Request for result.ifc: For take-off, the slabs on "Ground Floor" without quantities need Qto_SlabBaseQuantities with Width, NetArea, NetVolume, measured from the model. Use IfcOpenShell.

First a look at what the model holds.

```python
import ifcopenshell
import ifcopenshell.util.element
import ifcopenshell.util.unit

model = ifcopenshell.open("result.ifc")
print(model.schema)
for unit_type in ("LENGTHUNIT", "AREAUNIT", "VOLUMEUNIT"):
    print(unit_type, ifcopenshell.util.unit.calculate_unit_scale(model, unit_type))
storey = next(s for s in model.by_type("IfcBuildingStorey") if s.Name == "Ground Floor")
slabs = [e for e in ifcopenshell.util.element.get_decomposition(storey) if e.is_a("IfcSlab")]
for e in sorted(slabs, key=lambda e: e.id()):
    print(e.id(), e.is_a(), e.Name, list(ifcopenshell.util.element.get_psets(e, qtos_only=True)), sep=" | ")
```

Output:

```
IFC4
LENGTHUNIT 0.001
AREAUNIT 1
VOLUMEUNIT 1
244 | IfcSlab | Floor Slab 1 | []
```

```python
import ifcopenshell
import ifcopenshell.api.pset
import ifcopenshell.geom
import ifcopenshell.util.element
import ifcopenshell.util.shape
import ifcopenshell.util.unit

model = ifcopenshell.open("result.ifc")
unit_scale = ifcopenshell.util.unit.calculate_unit_scale(model)
area_scale = ifcopenshell.util.unit.calculate_unit_scale(model, "AREAUNIT")
volume_scale = ifcopenshell.util.unit.calculate_unit_scale(model, "VOLUMEUNIT")
settings = ifcopenshell.geom.settings()

storey = next(s for s in model.by_type("IfcBuildingStorey") if s.Name == "Ground Floor")
slabs = [e for e in ifcopenshell.util.element.get_decomposition(storey) if e.is_a("IfcSlab")]

for e in sorted(slabs, key=lambda e: e.id()):
    if ifcopenshell.util.element.get_psets(e, qtos_only=True, should_inherit=False):
        continue
    # Geometry comes back in metres, in the element's own axes.
    shape = ifcopenshell.geom.create_shape(settings, e)
    values = {
        "Width": ifcopenshell.util.shape.get_z(shape.geometry) / unit_scale,
        "NetArea": ifcopenshell.util.shape.get_footprint_area(shape.geometry) / area_scale,
        "NetVolume": ifcopenshell.util.shape.get_volume(shape.geometry) / volume_scale,
    }
    qto = ifcopenshell.api.pset.add_qto(model, product=e, name="Qto_SlabBaseQuantities")
    ifcopenshell.api.pset.edit_qto(model, qto=qto, properties=values)
    print(e.id(), {k: round(v, 3) for k, v in values.items()})

model.write("result_edited.ifc")
```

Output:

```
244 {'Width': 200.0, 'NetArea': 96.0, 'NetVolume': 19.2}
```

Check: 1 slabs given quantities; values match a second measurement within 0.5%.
